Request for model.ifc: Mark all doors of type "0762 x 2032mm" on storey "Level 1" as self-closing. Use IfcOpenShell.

First a look at what the model holds.

```python
import ifcopenshell
import ifcopenshell.util.element

model = ifcopenshell.open("model.ifc")
print(model.schema)
storey = next(s for s in model.by_type("IfcBuildingStorey") if s.Name == "Level 1")
doors = [e for e in ifcopenshell.util.element.get_decomposition(storey) if e.is_a("IfcDoor")]
seen = {}
for e in doors:
    element_type = ifcopenshell.util.element.get_type(e)
    key = (element_type.Name if element_type != e and element_type else None, ifcopenshell.util.element.get_pset(e, "Pset_DoorCommon", "SelfClosing"))
    seen[key] = seen.get(key, 0) + 1
for (name, value), count in sorted(seen.items(), key=str):
    print(count, "x", name, "|", value)
```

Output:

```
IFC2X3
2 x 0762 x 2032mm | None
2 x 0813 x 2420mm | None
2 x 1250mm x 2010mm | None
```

```python
import ifcopenshell
import ifcopenshell.api.pset
import ifcopenshell.util.element

model = ifcopenshell.open("model.ifc")

storey = next(s for s in model.by_type("IfcBuildingStorey") if s.Name == "Level 1")
doors = [e for e in ifcopenshell.util.element.get_decomposition(storey) if e.is_a("IfcDoor")]

count = 0
for e in doors:
    element_type = ifcopenshell.util.element.get_type(e)
    if element_type in (None, e) or element_type.Name != "0762 x 2032mm":
        continue
    # add_pset returns the element's existing set when there is one.
    pset = ifcopenshell.api.pset.add_pset(model, product=e, name="Pset_DoorCommon")
    ifcopenshell.api.pset.edit_pset(model, pset=pset, properties={"SelfClosing": True})
    count += 1

print(count, "doors updated")

model.write("model_updated.ifc")
```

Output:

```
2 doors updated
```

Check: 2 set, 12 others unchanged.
